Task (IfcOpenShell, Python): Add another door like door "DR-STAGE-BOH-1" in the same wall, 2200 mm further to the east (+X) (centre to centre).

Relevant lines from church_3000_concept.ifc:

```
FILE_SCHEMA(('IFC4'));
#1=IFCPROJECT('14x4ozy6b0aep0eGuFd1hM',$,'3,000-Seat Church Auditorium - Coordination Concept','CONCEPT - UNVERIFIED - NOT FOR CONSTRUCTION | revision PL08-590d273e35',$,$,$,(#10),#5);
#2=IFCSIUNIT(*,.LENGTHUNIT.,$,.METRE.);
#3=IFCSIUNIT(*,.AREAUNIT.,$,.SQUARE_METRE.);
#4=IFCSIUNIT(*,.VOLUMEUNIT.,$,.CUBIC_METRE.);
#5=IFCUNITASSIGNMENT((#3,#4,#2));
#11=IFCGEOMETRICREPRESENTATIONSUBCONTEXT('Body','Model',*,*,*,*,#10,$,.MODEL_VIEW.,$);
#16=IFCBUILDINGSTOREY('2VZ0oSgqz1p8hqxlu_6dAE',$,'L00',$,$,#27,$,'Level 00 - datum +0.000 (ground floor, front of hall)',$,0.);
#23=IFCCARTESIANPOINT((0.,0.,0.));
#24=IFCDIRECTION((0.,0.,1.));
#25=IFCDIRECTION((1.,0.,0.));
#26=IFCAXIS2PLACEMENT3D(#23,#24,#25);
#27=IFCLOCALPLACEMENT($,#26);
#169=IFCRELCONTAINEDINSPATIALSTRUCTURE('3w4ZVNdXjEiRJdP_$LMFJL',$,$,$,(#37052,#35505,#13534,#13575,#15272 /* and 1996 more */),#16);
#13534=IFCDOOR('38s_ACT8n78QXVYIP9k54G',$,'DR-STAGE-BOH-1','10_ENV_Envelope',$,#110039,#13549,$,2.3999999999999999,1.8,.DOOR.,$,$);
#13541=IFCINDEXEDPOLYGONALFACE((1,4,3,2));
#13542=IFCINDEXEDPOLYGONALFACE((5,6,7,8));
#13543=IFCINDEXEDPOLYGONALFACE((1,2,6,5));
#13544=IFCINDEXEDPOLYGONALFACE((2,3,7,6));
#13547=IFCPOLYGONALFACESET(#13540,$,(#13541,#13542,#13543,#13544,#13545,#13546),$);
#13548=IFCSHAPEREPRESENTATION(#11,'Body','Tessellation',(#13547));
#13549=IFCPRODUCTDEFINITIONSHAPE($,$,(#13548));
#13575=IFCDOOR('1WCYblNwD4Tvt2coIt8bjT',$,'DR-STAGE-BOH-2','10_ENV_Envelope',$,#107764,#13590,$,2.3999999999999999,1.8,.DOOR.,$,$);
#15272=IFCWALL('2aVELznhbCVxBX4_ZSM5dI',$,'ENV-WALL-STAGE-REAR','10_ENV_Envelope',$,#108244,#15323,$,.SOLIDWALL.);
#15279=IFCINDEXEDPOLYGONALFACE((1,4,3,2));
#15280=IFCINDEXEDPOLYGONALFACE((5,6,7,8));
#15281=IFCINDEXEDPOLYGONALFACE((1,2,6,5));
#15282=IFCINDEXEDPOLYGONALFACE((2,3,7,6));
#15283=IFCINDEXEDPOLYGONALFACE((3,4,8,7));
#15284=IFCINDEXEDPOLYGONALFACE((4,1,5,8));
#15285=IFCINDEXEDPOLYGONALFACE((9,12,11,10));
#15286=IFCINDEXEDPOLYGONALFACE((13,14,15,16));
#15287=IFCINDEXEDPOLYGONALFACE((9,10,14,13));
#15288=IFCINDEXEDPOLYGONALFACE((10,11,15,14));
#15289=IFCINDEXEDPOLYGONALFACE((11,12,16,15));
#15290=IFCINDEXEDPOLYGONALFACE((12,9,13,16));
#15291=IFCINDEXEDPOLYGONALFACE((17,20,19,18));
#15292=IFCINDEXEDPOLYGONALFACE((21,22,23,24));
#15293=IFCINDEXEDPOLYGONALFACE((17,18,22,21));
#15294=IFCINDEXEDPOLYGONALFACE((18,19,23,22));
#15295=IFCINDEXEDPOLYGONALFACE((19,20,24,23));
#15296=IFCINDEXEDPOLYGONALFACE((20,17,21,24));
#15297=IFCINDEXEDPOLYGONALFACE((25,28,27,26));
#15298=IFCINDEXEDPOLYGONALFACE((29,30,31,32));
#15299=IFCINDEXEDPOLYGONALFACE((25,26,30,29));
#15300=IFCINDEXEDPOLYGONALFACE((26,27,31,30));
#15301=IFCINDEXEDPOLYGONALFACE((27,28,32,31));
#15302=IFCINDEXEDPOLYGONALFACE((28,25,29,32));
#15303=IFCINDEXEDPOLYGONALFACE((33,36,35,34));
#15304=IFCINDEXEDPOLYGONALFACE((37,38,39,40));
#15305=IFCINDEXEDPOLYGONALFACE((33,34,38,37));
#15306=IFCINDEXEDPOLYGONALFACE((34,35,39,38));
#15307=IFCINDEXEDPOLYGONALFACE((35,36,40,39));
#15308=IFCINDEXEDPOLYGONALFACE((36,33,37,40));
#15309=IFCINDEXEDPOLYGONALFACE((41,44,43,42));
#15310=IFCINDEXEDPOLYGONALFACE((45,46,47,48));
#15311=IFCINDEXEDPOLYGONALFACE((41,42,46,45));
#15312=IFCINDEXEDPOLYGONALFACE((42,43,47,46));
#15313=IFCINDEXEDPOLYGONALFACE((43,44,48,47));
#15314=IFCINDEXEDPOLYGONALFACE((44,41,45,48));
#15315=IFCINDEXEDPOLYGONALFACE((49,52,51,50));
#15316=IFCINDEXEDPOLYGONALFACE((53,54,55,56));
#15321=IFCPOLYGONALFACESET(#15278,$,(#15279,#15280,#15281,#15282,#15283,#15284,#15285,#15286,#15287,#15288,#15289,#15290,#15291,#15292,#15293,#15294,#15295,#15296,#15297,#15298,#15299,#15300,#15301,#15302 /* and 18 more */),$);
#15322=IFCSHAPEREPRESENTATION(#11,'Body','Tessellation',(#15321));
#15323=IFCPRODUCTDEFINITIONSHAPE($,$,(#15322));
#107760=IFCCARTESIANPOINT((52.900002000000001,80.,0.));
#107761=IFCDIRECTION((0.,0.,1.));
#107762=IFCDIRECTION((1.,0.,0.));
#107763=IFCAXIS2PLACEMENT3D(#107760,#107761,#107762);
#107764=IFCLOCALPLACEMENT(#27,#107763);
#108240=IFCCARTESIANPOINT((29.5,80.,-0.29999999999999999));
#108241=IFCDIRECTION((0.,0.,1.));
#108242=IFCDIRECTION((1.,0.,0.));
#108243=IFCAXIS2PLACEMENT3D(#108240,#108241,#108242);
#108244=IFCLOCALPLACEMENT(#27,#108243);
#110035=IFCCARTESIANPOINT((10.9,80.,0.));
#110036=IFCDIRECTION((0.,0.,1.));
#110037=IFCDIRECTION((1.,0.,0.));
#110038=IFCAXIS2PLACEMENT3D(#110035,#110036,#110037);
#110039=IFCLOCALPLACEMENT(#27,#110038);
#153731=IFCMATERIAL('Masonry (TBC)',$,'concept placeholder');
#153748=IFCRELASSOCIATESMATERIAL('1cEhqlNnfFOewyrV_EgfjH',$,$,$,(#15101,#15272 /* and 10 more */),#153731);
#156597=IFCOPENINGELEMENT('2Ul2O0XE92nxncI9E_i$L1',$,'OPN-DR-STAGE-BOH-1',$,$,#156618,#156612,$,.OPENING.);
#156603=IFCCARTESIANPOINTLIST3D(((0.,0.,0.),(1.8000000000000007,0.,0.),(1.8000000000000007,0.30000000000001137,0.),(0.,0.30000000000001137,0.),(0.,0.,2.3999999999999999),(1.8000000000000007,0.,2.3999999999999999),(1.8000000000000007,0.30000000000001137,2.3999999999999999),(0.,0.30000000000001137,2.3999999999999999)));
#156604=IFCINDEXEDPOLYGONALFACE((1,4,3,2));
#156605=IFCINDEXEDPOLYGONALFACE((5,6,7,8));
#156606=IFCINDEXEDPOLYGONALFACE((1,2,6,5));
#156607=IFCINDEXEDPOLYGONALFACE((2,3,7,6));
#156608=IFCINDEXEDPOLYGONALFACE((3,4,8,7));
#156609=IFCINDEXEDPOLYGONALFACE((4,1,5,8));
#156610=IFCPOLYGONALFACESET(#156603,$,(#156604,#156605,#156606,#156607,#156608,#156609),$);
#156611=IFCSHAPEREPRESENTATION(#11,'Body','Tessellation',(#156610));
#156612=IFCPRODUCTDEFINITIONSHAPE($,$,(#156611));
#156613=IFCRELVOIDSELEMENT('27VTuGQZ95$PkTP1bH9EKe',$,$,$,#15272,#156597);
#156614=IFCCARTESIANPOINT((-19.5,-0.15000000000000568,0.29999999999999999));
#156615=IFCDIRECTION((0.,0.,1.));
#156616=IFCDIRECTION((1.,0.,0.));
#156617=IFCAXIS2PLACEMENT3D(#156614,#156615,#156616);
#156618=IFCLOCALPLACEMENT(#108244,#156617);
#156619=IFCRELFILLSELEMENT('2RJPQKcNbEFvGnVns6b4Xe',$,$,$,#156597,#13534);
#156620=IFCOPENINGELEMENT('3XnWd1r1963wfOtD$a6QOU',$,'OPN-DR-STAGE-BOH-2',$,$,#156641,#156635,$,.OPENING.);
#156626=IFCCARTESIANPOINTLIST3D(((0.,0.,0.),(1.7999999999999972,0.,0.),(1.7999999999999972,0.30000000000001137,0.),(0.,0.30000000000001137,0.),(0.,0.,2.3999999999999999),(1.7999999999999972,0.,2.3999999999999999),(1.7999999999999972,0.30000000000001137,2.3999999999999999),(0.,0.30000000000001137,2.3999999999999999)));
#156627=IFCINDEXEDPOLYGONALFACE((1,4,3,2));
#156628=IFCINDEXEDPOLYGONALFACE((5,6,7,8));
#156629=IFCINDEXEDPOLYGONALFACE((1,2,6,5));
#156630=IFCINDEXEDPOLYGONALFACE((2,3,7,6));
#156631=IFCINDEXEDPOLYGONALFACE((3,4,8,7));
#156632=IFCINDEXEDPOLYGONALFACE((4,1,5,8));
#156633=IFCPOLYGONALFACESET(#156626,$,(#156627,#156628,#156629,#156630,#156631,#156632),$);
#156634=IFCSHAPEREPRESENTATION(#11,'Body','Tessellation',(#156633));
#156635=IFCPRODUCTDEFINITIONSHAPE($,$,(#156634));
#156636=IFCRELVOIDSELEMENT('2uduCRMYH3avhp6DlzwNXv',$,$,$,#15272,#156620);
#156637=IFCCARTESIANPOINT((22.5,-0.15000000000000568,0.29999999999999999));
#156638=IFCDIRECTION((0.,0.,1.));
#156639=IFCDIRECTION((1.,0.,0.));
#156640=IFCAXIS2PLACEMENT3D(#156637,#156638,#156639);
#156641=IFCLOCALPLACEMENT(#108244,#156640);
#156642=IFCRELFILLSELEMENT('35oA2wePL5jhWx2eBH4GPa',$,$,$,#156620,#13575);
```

```python
import ifcopenshell
import ifcopenshell.api.feature
import ifcopenshell.api.geometry
import ifcopenshell.api.root
import ifcopenshell.geom
import ifcopenshell.util.element
import ifcopenshell.util.placement
import ifcopenshell.util.shape

model = ifcopenshell.open("church_3000_concept.ifc")
settings = ifcopenshell.geom.settings()


def volume(element):
    """Net volume in cubic metres, openings subtracted."""
    shape = ifcopenshell.geom.create_shape(settings, element)
    return ifcopenshell.util.shape.get_volume(shape.geometry)


door = model.by_guid("38s_ACT8n78QXVYIP9k54G")
opening = door.FillsVoids[0].RelatingOpeningElement
wall = opening.VoidsElements[0].RelatingBuildingElement
before = volume(wall)
shift = ifcopenshell.util.placement.get_local_placement(wall.ObjectPlacement)[:3, 0] * 2.2

# copy_class copies the void relationship, type, container and properties, but no geometry.
new_opening = ifcopenshell.api.root.copy_class(model, product=opening)
new_opening.Representation = ifcopenshell.util.element.copy_deep(
    model, opening.Representation, exclude=["IfcGeometricRepresentationContext", "IfcRepresentationMap"]
)
new_door = ifcopenshell.api.root.copy_class(model, product=door)
new_door.Representation = ifcopenshell.util.element.copy_deep(
    model, door.Representation, exclude=["IfcGeometricRepresentationContext", "IfcRepresentationMap"]
)
ifcopenshell.api.feature.add_filling(model, opening=new_opening, element=new_door)

for old, new in ((opening, new_opening), (door, new_door)):
    matrix = ifcopenshell.util.placement.get_local_placement(old.ObjectPlacement)
    matrix[:3, 3] += shift
    ifcopenshell.api.geometry.edit_object_placement(model, product=new, matrix=matrix, is_si=False)

after = volume(wall)

print(f"wall volume {before:.3f} -> {after:.3f} m3")

model.write("church_3000_concept_updated.ifc")
```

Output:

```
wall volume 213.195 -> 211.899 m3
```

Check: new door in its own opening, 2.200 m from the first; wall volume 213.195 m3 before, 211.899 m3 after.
